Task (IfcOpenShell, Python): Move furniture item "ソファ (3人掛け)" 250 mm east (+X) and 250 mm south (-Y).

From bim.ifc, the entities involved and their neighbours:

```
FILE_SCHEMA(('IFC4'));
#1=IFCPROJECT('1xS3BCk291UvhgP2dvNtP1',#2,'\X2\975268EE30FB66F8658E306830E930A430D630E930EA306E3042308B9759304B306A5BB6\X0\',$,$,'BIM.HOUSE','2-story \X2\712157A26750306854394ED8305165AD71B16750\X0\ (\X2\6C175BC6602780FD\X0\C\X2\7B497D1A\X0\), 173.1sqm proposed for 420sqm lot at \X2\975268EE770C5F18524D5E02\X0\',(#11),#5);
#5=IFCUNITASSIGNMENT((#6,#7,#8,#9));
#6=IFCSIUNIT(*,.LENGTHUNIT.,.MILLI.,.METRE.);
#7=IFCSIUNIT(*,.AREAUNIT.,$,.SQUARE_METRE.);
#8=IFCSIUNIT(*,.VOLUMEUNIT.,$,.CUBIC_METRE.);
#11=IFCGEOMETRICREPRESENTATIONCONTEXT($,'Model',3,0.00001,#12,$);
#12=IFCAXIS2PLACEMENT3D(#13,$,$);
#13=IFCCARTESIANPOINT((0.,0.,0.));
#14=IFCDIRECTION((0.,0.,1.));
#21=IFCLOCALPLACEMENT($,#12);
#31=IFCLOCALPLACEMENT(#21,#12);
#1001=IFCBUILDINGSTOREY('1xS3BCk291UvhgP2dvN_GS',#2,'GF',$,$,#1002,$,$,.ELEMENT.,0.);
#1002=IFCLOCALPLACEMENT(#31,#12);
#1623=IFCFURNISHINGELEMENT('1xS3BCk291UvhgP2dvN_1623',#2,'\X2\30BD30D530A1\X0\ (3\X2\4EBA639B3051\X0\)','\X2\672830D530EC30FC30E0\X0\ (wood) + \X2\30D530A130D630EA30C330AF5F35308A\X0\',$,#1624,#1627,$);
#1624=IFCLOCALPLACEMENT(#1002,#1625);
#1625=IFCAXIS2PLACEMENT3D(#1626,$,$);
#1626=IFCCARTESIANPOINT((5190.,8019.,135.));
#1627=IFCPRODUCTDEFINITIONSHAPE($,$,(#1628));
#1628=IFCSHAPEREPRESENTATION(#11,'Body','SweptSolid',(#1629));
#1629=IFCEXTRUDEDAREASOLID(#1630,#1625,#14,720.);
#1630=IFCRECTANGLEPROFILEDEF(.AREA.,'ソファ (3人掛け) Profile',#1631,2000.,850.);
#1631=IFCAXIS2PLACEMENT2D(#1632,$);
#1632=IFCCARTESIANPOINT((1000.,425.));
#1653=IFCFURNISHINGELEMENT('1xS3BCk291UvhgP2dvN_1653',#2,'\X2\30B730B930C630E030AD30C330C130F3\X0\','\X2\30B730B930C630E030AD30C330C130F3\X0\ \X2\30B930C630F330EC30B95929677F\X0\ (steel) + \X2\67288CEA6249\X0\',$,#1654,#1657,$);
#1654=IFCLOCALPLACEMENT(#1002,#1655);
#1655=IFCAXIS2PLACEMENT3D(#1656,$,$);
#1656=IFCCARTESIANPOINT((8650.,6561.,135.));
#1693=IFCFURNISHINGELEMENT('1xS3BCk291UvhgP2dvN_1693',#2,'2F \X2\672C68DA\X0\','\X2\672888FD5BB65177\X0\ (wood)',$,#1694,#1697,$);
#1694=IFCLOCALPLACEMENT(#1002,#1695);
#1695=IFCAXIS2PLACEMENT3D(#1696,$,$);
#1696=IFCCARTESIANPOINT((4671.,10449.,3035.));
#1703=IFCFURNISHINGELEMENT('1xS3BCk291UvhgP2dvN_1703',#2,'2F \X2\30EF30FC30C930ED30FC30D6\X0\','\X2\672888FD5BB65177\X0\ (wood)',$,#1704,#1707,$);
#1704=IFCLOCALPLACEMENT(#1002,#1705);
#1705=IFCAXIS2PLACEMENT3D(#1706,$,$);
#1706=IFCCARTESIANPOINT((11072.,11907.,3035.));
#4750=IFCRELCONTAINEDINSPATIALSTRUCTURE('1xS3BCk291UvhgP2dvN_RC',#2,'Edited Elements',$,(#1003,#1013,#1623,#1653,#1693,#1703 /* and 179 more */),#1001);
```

```python
import ifcopenshell
import ifcopenshell.api.geometry
import ifcopenshell.util.placement
import ifcopenshell.util.unit

model = ifcopenshell.open("bim.ifc")
unit_scale = ifcopenshell.util.unit.calculate_unit_scale(model)

item = model.by_guid("1xS3BCk291UvhgP2dvN_1623")
matrix = ifcopenshell.util.placement.get_local_placement(item.ObjectPlacement)
matrix[0, 3] += 0.25 / unit_scale
matrix[1, 3] -= 0.25 / unit_scale
ifcopenshell.api.geometry.edit_object_placement(model, product=item, matrix=matrix, is_si=False)

print(ifcopenshell.util.placement.get_local_placement(item.ObjectPlacement).round(3) + 0.0)

model.write("bim_edited.ifc")
```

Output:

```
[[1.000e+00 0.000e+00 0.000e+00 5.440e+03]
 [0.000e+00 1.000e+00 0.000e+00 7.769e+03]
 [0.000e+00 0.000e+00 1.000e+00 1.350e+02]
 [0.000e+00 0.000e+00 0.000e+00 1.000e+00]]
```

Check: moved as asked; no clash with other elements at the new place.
